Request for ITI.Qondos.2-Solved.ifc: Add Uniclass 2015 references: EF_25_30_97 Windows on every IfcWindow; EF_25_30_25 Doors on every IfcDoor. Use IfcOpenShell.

First a look at what the model holds.

```python
import ifcopenshell

model = ifcopenshell.open("ITI.Qondos.2-Solved.ifc")
print(model.schema)
print("classifications:", [c.Name for c in model.by_type("IfcClassification")])
for ifc_class in ("IfcDoor", "IfcRoof", "IfcStair", "IfcWall", "IfcWindow"):
    print(ifc_class, len(model.by_type(ifc_class)))
```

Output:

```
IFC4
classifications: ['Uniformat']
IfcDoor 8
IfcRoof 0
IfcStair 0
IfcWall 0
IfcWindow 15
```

```python
import ifcopenshell
import ifcopenshell.api.classification

model = ifcopenshell.open("ITI.Qondos.2-Solved.ifc")

system = ifcopenshell.api.classification.add_classification(model, classification="Uniclass 2015")

codes = {
    "IfcWindow": ("EF_25_30_97", "Windows"),
    "IfcDoor": ("EF_25_30_25", "Doors"),
}
for ifc_class, (code, name) in codes.items():
    products = model.by_type(ifc_class)
    ifcopenshell.api.classification.add_reference(
        model, products=products, classification=system, identification=code, name=name
    )
    print(code, len(products))

model.write("ITI.Qondos.2-Solved-out.ifc")
```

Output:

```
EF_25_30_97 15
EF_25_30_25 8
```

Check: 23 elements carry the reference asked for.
